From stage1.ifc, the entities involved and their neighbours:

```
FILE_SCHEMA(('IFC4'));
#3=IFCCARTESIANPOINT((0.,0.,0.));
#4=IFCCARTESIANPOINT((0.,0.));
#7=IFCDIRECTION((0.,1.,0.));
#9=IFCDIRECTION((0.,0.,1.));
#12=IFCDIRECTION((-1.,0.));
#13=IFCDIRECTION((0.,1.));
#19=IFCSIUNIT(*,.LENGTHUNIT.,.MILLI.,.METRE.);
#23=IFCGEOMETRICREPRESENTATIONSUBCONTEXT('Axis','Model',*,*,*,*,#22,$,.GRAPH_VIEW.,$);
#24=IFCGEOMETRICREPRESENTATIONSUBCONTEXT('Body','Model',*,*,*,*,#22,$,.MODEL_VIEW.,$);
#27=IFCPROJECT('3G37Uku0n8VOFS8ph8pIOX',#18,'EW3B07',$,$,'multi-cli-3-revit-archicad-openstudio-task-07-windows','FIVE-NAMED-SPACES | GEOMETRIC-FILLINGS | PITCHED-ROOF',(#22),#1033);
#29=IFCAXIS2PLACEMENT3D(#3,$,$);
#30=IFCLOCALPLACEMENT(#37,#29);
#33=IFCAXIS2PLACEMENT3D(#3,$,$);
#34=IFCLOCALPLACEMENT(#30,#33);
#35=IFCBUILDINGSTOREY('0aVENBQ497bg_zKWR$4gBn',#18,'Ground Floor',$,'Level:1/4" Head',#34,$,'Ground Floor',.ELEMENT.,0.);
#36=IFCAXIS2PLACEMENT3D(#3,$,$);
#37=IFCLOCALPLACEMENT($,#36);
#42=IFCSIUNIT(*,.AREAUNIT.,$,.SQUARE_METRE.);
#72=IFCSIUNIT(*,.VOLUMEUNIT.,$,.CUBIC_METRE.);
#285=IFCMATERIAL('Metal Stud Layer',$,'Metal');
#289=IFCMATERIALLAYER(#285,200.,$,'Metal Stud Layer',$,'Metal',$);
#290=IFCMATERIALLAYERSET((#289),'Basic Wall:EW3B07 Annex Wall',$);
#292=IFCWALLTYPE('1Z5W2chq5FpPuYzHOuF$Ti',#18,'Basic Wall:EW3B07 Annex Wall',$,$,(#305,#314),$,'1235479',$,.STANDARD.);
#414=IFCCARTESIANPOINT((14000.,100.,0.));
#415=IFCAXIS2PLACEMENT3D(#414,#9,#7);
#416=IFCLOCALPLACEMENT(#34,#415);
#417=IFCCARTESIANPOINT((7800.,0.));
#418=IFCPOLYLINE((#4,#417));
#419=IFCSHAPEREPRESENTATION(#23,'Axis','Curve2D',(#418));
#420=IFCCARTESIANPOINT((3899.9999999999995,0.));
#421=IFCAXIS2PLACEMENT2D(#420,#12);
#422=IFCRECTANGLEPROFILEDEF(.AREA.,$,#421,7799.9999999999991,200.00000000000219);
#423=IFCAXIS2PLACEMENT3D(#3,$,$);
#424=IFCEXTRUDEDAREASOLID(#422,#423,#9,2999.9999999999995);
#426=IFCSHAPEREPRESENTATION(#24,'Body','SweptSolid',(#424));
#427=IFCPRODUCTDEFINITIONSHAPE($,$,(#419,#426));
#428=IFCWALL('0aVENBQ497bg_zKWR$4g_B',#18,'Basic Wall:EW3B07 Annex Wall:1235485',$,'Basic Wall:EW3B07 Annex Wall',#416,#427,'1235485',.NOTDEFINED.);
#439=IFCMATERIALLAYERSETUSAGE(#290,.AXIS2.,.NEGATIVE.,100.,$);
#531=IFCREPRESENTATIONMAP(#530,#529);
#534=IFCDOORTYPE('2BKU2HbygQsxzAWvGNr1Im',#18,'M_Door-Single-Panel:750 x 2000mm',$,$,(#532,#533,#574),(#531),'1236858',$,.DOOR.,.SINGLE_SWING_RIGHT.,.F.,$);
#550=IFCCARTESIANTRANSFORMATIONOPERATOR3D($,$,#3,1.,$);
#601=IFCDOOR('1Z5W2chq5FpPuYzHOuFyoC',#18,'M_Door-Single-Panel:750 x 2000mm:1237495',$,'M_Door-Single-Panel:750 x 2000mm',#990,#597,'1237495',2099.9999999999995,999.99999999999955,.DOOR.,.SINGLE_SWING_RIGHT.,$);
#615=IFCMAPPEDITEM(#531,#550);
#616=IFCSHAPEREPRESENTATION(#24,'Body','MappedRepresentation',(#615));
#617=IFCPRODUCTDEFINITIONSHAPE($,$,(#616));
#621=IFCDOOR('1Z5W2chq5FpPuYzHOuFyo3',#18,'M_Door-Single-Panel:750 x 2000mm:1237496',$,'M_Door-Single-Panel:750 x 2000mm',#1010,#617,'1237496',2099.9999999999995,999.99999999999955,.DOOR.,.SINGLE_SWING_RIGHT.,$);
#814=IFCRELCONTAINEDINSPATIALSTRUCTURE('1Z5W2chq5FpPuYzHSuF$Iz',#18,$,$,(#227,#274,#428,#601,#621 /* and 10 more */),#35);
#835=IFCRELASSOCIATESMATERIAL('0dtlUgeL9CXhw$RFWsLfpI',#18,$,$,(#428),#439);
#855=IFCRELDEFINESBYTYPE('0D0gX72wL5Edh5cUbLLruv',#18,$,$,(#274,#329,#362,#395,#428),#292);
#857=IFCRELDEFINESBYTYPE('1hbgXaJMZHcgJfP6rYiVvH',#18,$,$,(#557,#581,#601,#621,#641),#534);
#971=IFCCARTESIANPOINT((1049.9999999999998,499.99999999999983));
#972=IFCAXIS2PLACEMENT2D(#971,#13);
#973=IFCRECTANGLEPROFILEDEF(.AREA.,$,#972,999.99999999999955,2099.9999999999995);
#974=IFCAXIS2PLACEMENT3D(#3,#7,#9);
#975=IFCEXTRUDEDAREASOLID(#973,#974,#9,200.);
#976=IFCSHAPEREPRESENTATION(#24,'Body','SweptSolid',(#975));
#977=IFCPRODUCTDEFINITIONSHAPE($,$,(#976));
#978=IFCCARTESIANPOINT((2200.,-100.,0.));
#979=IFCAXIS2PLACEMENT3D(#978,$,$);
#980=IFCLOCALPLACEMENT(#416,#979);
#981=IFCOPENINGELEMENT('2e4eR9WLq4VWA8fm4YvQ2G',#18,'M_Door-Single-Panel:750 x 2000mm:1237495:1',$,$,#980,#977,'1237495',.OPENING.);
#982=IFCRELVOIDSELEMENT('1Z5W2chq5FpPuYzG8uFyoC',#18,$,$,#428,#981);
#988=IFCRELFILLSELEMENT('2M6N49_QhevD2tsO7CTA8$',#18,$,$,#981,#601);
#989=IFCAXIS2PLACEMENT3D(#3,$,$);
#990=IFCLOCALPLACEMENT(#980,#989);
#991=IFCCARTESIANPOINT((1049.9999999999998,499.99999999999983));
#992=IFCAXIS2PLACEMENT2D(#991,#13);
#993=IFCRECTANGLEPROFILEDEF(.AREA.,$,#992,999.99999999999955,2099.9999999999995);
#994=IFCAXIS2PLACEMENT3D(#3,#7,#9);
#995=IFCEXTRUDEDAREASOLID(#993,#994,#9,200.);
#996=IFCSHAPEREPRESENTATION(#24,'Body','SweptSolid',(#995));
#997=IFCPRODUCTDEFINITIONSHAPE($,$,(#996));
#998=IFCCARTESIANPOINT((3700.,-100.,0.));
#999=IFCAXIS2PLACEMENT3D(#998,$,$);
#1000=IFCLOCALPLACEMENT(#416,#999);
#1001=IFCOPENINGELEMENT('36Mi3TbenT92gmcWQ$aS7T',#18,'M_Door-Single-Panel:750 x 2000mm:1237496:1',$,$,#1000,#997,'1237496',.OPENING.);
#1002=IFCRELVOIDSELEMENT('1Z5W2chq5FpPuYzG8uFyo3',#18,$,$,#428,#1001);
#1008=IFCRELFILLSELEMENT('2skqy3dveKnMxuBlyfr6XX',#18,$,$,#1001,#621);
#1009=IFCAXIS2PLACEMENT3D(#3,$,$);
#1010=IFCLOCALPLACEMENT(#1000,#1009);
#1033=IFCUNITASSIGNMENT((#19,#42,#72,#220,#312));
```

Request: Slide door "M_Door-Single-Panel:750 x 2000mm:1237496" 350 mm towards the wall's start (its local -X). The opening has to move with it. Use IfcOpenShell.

```python
import ifcopenshell
import ifcopenshell.api.geometry
import ifcopenshell.util.placement
import ifcopenshell.util.unit

model = ifcopenshell.open("stage1.ifc")
unit_scale = ifcopenshell.util.unit.calculate_unit_scale(model)

door = model.by_id(621)
opening = door.FillsVoids[0].RelatingOpeningElement
wall = opening.VoidsElements[0].RelatingBuildingElement

wall_matrix = ifcopenshell.util.placement.get_local_placement(wall.ObjectPlacement)
shift = wall_matrix[:3, 0] * -0.35 / unit_scale
before = ifcopenshell.util.placement.get_local_placement(door.ObjectPlacement)[:3, 3].copy()

# The door is placed relative to its opening, so it follows when the opening moves.
matrix = ifcopenshell.util.placement.get_local_placement(opening.ObjectPlacement)
matrix[:3, 3] += shift
ifcopenshell.api.geometry.edit_object_placement(
    model, product=opening, matrix=matrix, is_si=False, should_transform_children=True
)

after = ifcopenshell.util.placement.get_local_placement(door.ObjectPlacement)[:3, 3]
print("door moved by", (after - before).round(3) + 0.0)

model.write("stage1_updated.ifc")
```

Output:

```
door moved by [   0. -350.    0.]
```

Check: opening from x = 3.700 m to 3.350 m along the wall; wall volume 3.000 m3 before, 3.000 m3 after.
